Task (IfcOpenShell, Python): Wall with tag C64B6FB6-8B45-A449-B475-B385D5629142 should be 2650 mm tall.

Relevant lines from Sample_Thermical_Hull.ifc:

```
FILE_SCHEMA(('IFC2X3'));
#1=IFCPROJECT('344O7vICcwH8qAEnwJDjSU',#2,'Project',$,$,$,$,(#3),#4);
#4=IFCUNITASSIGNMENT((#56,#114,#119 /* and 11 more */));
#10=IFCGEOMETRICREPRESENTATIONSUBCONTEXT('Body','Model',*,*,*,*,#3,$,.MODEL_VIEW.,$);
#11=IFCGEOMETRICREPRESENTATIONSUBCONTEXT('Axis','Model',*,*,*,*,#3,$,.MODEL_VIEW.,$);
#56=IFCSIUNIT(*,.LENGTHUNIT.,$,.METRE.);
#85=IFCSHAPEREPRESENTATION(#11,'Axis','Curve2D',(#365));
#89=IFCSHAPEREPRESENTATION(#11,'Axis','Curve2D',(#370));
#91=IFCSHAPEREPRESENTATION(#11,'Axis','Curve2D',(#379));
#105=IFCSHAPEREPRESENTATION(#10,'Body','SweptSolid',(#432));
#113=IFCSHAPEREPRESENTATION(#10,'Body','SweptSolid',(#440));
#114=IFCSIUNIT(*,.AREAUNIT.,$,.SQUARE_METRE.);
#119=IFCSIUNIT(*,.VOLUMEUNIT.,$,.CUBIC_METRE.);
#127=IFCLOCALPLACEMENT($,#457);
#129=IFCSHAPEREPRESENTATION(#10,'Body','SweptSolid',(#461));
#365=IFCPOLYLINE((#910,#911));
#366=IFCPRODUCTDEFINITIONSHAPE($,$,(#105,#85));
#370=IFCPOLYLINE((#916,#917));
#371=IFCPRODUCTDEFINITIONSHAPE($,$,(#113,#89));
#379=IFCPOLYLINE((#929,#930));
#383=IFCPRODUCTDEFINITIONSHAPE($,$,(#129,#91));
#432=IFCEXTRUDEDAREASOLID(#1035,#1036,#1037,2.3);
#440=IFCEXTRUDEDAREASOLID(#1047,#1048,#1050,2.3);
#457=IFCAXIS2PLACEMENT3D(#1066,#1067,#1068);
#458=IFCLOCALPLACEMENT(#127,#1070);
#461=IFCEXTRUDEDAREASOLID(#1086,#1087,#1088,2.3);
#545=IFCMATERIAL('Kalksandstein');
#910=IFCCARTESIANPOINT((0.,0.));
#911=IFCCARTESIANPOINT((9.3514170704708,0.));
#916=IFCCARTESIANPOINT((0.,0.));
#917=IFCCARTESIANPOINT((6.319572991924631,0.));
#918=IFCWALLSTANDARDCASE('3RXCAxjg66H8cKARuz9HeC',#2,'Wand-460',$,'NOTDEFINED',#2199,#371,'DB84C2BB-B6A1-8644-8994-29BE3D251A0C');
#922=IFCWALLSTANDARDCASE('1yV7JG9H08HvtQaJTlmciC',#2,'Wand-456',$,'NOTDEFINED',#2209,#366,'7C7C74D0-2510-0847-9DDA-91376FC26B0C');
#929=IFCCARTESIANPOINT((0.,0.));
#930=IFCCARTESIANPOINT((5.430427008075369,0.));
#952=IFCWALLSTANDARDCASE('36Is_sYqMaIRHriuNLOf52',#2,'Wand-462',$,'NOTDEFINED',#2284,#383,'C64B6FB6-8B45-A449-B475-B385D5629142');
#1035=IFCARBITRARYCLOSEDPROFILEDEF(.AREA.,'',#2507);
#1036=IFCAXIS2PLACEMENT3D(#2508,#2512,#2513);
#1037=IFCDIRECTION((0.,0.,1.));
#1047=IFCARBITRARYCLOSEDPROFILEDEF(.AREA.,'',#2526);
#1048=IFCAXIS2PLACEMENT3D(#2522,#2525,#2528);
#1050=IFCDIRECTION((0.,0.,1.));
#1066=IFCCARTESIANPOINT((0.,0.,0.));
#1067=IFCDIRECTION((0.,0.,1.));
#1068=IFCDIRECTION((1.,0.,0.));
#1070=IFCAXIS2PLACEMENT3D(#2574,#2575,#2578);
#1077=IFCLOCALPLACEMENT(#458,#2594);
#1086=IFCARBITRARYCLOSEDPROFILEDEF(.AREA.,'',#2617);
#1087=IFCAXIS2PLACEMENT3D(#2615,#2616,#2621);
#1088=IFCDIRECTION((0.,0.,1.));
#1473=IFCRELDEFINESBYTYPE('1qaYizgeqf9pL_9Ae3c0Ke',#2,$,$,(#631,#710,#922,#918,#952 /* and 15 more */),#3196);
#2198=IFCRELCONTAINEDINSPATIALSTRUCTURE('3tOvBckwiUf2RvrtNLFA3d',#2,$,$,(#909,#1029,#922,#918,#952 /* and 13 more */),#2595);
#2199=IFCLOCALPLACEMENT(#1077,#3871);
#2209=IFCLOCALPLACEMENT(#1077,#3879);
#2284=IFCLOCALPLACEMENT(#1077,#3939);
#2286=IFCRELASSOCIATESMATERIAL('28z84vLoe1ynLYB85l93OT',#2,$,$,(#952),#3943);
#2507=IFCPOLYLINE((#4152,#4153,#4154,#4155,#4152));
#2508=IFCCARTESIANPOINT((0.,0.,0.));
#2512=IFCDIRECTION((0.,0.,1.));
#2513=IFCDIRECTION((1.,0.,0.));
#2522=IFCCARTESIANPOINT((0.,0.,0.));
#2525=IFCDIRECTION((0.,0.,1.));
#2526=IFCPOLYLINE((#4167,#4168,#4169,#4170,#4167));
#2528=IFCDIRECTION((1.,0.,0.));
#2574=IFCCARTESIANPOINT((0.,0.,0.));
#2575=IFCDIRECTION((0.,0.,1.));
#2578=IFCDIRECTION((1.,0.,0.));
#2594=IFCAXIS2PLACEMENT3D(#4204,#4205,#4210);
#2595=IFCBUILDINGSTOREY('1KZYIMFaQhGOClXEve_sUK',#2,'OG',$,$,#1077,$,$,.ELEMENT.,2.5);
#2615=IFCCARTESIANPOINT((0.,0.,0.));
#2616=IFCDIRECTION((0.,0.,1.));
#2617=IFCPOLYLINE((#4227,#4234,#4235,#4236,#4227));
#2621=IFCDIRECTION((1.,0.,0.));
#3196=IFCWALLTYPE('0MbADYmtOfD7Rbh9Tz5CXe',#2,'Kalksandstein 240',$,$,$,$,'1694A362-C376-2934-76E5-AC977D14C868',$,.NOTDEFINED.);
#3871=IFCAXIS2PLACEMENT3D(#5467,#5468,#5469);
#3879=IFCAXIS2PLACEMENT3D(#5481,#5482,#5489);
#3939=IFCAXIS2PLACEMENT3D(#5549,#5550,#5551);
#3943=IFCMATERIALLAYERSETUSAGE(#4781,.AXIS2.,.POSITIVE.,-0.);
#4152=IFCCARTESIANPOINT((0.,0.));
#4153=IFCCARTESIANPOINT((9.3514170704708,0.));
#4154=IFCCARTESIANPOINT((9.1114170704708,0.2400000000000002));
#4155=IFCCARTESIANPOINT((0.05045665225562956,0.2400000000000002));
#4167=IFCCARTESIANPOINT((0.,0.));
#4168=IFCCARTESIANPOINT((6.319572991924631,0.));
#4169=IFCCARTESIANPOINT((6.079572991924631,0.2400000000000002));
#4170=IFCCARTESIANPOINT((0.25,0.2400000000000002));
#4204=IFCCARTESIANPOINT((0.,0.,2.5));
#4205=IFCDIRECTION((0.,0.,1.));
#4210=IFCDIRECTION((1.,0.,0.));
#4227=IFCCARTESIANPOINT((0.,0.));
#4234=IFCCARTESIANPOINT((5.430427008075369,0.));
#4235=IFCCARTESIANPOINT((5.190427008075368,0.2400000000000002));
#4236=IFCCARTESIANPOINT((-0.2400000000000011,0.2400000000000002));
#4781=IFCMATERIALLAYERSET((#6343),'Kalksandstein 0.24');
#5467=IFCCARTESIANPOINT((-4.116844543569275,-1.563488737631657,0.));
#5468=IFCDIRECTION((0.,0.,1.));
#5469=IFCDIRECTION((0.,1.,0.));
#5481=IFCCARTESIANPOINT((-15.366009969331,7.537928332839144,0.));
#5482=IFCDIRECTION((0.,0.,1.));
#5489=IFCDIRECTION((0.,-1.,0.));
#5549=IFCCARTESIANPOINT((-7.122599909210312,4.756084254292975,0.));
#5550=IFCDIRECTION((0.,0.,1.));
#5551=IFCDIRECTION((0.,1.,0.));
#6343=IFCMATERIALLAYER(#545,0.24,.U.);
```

```python
import ifcopenshell
import ifcopenshell.geom
import ifcopenshell.util.representation
import ifcopenshell.util.shape
import ifcopenshell.util.unit

model = ifcopenshell.open("Sample_Thermical_Hull.ifc")
unit_scale = ifcopenshell.util.unit.calculate_unit_scale(model)
settings = ifcopenshell.geom.settings()


def volume(element):
    """Net volume in cubic metres, openings subtracted."""
    shape = ifcopenshell.geom.create_shape(settings, element)
    return ifcopenshell.util.shape.get_volume(shape.geometry)


wall = model.by_guid("36Is_sYqMaIRHriuNLOf52")
before = volume(wall)

body = ifcopenshell.util.representation.get_representation(wall, "Model", "Body")
solid = body.Items[0]
old_height = solid.Depth
solid.Depth = 2.65 / unit_scale
after = volume(wall)

print(f"height {old_height:g} -> {solid.Depth:g}, volume {before:.3f} -> {after:.3f} m3")

model.write("Sample_Thermical_Hull_v2.ifc")
```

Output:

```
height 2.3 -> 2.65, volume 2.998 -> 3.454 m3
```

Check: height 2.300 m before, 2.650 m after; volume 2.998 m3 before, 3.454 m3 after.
